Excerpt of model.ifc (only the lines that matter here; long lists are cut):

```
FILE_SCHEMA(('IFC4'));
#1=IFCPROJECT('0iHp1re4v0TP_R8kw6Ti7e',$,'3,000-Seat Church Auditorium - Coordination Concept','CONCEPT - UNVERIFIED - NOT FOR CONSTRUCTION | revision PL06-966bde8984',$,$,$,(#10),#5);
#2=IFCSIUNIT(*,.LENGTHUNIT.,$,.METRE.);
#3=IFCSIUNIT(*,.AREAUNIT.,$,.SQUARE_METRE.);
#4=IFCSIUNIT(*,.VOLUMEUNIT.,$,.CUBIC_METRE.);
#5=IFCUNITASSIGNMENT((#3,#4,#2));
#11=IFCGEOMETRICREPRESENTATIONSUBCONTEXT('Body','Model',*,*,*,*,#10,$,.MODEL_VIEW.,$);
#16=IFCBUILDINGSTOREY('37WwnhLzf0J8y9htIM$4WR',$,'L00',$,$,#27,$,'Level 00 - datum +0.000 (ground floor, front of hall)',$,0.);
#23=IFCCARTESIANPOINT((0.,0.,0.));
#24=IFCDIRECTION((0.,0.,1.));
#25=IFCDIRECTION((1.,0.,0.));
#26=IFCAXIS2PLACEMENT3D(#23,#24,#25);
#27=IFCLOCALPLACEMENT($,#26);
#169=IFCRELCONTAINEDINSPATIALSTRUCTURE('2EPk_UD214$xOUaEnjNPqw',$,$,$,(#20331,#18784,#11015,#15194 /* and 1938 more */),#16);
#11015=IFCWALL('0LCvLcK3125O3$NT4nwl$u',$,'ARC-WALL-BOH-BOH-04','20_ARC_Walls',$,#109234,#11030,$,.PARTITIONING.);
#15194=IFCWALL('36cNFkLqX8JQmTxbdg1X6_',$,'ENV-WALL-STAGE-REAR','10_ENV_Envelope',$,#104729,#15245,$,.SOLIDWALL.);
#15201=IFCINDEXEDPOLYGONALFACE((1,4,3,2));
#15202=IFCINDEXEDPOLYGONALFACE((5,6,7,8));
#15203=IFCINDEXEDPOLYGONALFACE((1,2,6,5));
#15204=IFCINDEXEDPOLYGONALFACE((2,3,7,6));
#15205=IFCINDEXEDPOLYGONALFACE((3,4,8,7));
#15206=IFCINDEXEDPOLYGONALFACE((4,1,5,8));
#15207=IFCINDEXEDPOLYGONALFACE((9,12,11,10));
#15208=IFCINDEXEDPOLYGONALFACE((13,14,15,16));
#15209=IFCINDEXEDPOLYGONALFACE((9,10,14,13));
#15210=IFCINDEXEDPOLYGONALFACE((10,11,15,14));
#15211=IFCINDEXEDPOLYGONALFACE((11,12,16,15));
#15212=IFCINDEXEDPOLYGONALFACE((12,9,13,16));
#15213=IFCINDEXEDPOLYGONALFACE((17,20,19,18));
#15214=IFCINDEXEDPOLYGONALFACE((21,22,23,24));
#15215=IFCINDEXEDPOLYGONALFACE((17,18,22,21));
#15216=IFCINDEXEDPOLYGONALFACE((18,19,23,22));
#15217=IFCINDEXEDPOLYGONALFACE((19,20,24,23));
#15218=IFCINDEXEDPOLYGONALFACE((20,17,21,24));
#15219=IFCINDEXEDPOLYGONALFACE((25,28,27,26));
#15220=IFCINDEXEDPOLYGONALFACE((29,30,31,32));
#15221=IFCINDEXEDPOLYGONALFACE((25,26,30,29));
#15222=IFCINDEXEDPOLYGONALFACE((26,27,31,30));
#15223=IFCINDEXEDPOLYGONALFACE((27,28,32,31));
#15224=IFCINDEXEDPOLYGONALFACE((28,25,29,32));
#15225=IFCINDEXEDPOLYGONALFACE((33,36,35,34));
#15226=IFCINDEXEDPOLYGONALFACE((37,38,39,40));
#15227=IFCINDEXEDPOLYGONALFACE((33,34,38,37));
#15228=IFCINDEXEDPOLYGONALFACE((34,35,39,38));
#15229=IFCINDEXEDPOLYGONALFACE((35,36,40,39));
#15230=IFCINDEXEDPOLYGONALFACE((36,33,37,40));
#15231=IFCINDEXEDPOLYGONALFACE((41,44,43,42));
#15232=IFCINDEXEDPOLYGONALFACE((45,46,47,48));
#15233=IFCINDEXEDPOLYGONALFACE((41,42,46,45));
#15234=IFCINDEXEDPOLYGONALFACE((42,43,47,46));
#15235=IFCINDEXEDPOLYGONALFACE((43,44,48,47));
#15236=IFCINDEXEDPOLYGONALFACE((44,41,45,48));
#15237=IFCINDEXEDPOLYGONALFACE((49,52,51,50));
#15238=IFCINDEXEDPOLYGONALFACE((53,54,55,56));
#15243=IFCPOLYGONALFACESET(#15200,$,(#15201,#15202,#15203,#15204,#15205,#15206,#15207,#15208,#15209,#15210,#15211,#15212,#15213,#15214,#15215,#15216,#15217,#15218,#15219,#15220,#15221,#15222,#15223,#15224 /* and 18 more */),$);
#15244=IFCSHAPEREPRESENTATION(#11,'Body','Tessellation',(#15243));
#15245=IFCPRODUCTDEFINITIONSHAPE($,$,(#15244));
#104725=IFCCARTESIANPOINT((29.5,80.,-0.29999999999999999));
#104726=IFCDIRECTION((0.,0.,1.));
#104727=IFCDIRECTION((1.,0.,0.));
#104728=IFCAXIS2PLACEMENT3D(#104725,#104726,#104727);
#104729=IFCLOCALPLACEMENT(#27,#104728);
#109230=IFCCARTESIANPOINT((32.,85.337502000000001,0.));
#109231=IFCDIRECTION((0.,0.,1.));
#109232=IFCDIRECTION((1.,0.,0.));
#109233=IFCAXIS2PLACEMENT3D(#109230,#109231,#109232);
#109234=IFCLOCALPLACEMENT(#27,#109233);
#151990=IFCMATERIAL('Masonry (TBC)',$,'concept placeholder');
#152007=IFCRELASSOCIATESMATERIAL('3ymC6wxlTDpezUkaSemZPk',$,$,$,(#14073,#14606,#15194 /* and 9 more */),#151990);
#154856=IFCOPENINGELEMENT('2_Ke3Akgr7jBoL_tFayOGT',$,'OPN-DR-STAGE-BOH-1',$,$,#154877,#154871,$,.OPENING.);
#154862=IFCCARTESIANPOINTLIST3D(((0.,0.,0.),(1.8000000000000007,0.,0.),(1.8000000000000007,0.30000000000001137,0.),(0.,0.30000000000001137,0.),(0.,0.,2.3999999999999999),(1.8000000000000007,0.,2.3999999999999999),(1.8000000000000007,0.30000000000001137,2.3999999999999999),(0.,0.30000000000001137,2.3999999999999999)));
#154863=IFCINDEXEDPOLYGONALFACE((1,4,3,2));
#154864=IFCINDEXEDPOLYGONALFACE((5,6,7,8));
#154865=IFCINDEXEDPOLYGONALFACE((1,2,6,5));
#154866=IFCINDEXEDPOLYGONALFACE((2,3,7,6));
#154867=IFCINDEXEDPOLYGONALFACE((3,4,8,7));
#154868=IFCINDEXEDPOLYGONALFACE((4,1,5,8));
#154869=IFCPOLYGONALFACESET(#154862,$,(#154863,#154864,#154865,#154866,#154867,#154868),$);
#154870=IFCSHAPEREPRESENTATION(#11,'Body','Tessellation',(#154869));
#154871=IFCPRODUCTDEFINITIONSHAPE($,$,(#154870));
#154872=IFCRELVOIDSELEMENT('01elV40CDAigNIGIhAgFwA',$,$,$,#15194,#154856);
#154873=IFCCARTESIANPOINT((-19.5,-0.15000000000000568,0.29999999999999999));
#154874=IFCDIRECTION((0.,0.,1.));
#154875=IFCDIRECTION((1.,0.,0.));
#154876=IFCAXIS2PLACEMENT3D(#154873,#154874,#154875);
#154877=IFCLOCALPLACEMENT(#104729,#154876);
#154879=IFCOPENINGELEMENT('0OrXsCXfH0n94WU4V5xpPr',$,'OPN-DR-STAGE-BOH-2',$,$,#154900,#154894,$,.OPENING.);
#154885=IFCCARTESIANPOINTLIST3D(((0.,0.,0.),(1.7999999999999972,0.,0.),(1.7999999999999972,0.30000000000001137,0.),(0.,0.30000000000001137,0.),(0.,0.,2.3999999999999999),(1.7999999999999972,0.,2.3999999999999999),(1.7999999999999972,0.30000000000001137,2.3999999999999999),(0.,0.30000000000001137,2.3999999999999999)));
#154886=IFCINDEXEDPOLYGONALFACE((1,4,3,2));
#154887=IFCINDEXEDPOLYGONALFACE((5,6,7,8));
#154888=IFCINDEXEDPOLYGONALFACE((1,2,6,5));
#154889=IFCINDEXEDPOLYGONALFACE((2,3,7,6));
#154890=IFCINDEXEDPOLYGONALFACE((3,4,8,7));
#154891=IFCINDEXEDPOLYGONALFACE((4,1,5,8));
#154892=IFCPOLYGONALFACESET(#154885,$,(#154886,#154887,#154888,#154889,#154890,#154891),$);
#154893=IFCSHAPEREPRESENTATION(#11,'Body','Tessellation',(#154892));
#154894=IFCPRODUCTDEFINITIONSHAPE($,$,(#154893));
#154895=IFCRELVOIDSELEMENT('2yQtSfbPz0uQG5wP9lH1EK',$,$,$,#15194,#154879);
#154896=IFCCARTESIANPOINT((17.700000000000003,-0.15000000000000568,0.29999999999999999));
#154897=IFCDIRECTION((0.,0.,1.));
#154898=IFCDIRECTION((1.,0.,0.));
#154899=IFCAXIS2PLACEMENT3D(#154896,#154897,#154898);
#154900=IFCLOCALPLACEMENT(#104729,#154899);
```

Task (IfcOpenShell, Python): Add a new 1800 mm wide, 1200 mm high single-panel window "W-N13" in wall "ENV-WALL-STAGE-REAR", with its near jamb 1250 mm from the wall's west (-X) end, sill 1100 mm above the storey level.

```python
import numpy as np
import ifcopenshell
import ifcopenshell.api.feature
import ifcopenshell.api.geometry
import ifcopenshell.api.root
import ifcopenshell.api.spatial
import ifcopenshell.geom
import ifcopenshell.util.element
import ifcopenshell.util.placement
import ifcopenshell.util.representation
import ifcopenshell.util.shape
import ifcopenshell.util.unit

model = ifcopenshell.open("model.ifc")
unit_scale = ifcopenshell.util.unit.calculate_unit_scale(model)
settings = ifcopenshell.geom.settings()


def volume(element):
    """Net volume in cubic metres, openings subtracted."""
    shape = ifcopenshell.geom.create_shape(settings, element)
    return ifcopenshell.util.shape.get_volume(shape.geometry)


wall = model.by_guid("36cNFkLqX8JQmTxbdg1X6_")
storey = ifcopenshell.util.element.get_container(wall, ifc_class="IfcBuildingStorey")
context = ifcopenshell.util.representation.get_context(model, "Model", "Body", "MODEL_VIEW")
before = volume(wall)

width, height, from_end, sill = 1.8, 1.2, 1.25, 1.1  # metres

# The wall runs along its own X axis, and the end named is its -X end.
wall_shape = ifcopenshell.geom.create_shape(settings, wall)
x, y, z = ifcopenshell.util.shape.get_vertices(wall_shape.geometry).T
start = x.min() + from_end
face, thickness = float(y.min()), float(y.max() - y.min())
wall_matrix = ifcopenshell.util.placement.get_local_placement(wall.ObjectPlacement)
level = ifcopenshell.util.placement.get_local_placement(storey.ObjectPlacement)[2, 3]


def in_wall(x, y):
    """Placement at x, y metres in the wall's axes, at sill height."""
    matrix = wall_matrix.copy()
    matrix[:, 3] = wall_matrix @ np.array([x / unit_scale, y / unit_scale, 0.0, 1.0])
    matrix[2, 3] = level + sill / unit_scale
    return matrix


# Opening: a box that overshoots both wall faces by 50 mm.
opening = ifcopenshell.api.root.create_entity(model, ifc_class="IfcOpeningElement", predefined_type="OPENING")
box = ifcopenshell.api.geometry.add_wall_representation(
    model, context=context, length=width, height=height, thickness=thickness + 0.1
)
ifcopenshell.api.geometry.assign_representation(model, product=opening, representation=box)
ifcopenshell.api.geometry.edit_object_placement(model, product=opening, matrix=in_wall(start, face - 0.05), is_si=False)
ifcopenshell.api.feature.add_feature(model, feature=opening, element=wall)

window = ifcopenshell.api.root.create_entity(model, ifc_class="IfcWindow", name="W-N13", predefined_type="WINDOW")
window.OverallWidth, window.OverallHeight = width / unit_scale, height / unit_scale
window.PartitioningType = "SINGLE_PANEL"
body = ifcopenshell.api.geometry.add_window_representation(
    model,
    context=context,
    overall_width=window.OverallWidth,
    overall_height=window.OverallHeight,
    partition_type="SINGLE_PANEL",
)
ifcopenshell.api.geometry.assign_representation(model, product=window, representation=body)
ifcopenshell.api.spatial.assign_container(model, products=[window], relating_structure=storey)
ifcopenshell.api.feature.add_filling(model, opening=opening, element=window)

# Centre the window in the wall's thickness.
ifcopenshell.api.geometry.edit_object_placement(model, product=window, matrix=in_wall(start, face), is_si=False)
window_shape = ifcopenshell.geom.create_shape(settings, window)
depth = ifcopenshell.util.shape.get_vertices(window_shape.geometry)[:, 1]
offset = face + thickness / 2 - (depth.min() + depth.max()) / 2
ifcopenshell.api.geometry.edit_object_placement(model, product=window, matrix=in_wall(start, offset), is_si=False)

after = volume(wall)

print(f"wall volume {before:.3f} -> {after:.3f} m3")

model.write("model_updated.ifc")
```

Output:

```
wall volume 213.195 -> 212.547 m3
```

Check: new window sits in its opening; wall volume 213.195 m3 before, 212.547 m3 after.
